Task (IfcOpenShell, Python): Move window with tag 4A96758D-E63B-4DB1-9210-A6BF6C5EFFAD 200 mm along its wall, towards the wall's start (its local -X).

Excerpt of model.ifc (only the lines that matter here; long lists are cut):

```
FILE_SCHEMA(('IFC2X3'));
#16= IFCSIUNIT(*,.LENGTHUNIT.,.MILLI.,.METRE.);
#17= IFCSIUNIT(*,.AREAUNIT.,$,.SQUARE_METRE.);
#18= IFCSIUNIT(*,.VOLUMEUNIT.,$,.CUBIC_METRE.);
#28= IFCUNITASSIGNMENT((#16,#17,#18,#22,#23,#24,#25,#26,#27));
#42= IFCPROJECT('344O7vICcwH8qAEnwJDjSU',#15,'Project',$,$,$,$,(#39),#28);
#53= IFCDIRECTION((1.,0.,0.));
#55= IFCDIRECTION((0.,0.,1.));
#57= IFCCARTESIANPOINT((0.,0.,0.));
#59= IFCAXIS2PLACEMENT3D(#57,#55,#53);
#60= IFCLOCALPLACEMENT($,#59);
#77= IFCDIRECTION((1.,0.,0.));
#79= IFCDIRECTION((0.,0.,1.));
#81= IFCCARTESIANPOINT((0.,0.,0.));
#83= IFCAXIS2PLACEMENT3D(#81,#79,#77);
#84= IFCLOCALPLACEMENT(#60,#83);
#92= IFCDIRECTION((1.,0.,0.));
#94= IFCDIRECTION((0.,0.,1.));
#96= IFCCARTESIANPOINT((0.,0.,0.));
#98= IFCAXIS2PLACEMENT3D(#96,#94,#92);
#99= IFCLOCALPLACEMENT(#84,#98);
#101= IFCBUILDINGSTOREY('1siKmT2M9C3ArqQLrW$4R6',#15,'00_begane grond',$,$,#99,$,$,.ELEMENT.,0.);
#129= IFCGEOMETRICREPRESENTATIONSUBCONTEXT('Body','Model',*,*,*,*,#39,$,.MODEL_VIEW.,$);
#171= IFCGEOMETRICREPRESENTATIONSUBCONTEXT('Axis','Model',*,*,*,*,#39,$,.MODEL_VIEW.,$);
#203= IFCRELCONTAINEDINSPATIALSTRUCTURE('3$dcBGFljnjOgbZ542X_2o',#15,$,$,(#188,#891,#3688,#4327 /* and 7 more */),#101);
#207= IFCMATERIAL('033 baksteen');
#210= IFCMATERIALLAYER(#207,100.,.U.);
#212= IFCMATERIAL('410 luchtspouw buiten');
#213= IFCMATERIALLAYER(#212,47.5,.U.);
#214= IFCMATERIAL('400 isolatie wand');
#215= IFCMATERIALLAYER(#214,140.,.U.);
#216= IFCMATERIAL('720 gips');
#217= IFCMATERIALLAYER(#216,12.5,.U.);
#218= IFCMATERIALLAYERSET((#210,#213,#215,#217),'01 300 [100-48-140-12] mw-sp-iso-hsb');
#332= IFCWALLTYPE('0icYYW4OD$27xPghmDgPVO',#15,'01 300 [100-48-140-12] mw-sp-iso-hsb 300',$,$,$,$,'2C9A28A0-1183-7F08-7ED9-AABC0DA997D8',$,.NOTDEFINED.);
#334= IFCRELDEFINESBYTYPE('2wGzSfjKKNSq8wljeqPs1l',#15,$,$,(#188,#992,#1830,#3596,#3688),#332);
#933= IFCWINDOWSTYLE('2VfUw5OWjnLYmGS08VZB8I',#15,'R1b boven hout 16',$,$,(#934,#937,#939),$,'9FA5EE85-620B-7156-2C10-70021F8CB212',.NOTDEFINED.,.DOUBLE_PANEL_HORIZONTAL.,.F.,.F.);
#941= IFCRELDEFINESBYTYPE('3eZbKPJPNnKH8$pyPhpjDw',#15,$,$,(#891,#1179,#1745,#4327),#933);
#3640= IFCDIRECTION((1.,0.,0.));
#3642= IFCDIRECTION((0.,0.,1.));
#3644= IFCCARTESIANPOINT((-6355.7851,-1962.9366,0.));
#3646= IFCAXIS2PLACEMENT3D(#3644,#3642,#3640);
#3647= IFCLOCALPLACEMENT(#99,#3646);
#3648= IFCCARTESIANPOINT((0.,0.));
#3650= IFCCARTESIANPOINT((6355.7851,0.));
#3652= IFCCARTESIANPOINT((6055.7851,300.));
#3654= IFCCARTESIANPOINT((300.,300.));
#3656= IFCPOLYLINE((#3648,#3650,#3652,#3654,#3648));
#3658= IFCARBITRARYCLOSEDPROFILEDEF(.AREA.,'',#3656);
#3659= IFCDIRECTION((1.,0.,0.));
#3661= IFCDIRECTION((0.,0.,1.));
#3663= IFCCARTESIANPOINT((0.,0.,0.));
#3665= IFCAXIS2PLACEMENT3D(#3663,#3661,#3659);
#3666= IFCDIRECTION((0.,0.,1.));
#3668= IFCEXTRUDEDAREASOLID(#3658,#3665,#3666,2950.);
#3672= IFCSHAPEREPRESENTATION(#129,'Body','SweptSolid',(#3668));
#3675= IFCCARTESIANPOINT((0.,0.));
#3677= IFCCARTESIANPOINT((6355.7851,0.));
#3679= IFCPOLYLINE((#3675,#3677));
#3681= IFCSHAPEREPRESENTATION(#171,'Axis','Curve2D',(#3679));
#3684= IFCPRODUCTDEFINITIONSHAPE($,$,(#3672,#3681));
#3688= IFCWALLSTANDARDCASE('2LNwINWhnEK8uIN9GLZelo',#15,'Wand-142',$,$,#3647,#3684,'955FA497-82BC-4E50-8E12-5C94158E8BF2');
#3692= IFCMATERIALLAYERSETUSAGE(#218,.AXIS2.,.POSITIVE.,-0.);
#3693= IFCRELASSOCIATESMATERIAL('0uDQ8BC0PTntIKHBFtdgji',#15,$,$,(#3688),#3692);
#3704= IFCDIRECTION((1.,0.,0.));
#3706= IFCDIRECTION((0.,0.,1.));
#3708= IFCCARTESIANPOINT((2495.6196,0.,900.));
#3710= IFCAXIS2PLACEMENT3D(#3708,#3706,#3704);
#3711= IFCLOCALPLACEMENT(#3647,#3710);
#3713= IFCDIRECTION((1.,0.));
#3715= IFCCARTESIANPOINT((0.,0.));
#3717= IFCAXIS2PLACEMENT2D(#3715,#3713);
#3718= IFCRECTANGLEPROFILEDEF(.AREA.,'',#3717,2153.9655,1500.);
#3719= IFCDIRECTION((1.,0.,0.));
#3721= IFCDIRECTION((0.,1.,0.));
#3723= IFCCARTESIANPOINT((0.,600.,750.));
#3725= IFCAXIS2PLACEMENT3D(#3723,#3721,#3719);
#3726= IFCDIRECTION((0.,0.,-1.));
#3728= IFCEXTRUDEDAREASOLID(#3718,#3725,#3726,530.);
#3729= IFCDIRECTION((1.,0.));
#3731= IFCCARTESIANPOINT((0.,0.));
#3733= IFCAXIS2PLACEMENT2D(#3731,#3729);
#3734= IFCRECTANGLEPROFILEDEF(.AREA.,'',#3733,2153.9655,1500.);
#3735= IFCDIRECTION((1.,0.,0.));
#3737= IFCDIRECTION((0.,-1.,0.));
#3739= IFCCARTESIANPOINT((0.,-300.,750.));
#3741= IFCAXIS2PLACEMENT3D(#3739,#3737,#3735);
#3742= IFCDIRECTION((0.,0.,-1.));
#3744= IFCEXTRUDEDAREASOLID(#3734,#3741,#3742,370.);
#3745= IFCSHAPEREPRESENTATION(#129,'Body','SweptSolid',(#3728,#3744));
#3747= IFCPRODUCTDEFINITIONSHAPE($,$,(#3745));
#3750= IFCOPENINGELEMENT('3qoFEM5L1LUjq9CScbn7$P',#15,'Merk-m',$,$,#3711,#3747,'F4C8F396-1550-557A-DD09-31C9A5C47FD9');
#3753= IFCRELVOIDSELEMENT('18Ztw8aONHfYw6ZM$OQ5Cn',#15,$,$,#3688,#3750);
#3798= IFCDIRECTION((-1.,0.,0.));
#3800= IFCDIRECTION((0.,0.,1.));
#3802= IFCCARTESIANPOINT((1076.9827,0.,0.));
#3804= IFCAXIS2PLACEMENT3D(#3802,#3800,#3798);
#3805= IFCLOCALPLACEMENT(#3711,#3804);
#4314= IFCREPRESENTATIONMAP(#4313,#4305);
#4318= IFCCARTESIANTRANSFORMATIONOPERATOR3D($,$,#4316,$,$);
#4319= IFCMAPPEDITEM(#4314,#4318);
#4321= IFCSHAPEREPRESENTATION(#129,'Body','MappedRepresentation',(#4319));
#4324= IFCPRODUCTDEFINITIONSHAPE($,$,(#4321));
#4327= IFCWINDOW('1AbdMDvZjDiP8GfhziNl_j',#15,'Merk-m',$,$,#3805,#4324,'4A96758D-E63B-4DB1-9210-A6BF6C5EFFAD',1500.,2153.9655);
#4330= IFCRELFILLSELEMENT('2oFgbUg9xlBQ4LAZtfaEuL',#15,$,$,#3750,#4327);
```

```python
import ifcopenshell
import ifcopenshell.api.geometry
import ifcopenshell.util.placement
import ifcopenshell.util.unit

model = ifcopenshell.open("model.ifc")
unit_scale = ifcopenshell.util.unit.calculate_unit_scale(model)

window = model.by_guid("1AbdMDvZjDiP8GfhziNl_j")
opening = window.FillsVoids[0].RelatingOpeningElement
wall = opening.VoidsElements[0].RelatingBuildingElement

wall_matrix = ifcopenshell.util.placement.get_local_placement(wall.ObjectPlacement)
shift = wall_matrix[:3, 0] * -0.2 / unit_scale
before = ifcopenshell.util.placement.get_local_placement(window.ObjectPlacement)[:3, 3].copy()

# The window is placed relative to its opening, so it follows when the opening moves.
matrix = ifcopenshell.util.placement.get_local_placement(opening.ObjectPlacement)
matrix[:3, 3] += shift
ifcopenshell.api.geometry.edit_object_placement(
    model, product=opening, matrix=matrix, is_si=False, should_transform_children=True
)

after = ifcopenshell.util.placement.get_local_placement(window.ObjectPlacement)[:3, 3]
print("window moved by", (after - before).round(3) + 0.0)

model.write("model_rev.ifc")
```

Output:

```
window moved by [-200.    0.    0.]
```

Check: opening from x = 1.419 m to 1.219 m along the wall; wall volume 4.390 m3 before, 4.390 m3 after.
